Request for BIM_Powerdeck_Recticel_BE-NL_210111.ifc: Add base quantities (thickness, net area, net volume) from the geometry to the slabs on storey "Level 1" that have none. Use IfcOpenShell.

First a look at what the model holds.

```python
import ifcopenshell
import ifcopenshell.util.element
import ifcopenshell.util.unit

model = ifcopenshell.open("BIM_Powerdeck_Recticel_BE-NL_210111.ifc")
print(model.schema)
for unit_type in ("LENGTHUNIT", "AREAUNIT", "VOLUMEUNIT"):
    print(unit_type, ifcopenshell.util.unit.calculate_unit_scale(model, unit_type))
storey = next(s for s in model.by_type("IfcBuildingStorey") if s.Name == "Level 1")
slabs = [e for e in ifcopenshell.util.element.get_decomposition(storey) if e.is_a("IfcSlab")]
for e in sorted(slabs, key=lambda e: e.id()):
    print(e.id(), e.is_a(), e.Name, list(ifcopenshell.util.element.get_psets(e, qtos_only=True)), sep=" | ")
```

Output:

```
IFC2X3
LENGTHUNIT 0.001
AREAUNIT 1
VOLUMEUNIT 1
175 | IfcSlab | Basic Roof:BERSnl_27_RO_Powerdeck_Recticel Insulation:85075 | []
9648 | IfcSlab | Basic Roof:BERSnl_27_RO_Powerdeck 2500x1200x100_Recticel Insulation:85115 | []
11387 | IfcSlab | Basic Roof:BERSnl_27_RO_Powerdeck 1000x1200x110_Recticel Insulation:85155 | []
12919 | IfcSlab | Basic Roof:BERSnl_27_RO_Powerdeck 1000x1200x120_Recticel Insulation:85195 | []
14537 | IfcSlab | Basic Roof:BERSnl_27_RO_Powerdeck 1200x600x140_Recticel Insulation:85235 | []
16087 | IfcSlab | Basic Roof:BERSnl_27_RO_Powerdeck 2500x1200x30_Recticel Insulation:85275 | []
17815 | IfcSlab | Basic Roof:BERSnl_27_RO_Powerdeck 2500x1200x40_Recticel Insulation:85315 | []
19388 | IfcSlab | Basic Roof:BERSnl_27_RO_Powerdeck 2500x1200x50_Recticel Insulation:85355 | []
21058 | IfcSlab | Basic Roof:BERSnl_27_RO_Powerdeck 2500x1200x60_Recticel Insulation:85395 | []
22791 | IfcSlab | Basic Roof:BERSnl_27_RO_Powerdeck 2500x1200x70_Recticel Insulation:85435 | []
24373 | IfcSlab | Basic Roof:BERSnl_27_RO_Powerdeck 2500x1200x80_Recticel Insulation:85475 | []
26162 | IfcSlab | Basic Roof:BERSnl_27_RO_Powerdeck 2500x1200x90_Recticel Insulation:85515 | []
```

```python
import ifcopenshell
import ifcopenshell.api.pset
import ifcopenshell.geom
import ifcopenshell.util.element
import ifcopenshell.util.shape
import ifcopenshell.util.unit

model = ifcopenshell.open("BIM_Powerdeck_Recticel_BE-NL_210111.ifc")
unit_scale = ifcopenshell.util.unit.calculate_unit_scale(model)
area_scale = ifcopenshell.util.unit.calculate_unit_scale(model, "AREAUNIT")
volume_scale = ifcopenshell.util.unit.calculate_unit_scale(model, "VOLUMEUNIT")
settings = ifcopenshell.geom.settings()

storey = next(s for s in model.by_type("IfcBuildingStorey") if s.Name == "Level 1")
slabs = [e for e in ifcopenshell.util.element.get_decomposition(storey) if e.is_a("IfcSlab")]

for e in sorted(slabs, key=lambda e: e.id()):
    if ifcopenshell.util.element.get_psets(e, qtos_only=True, should_inherit=False):
        continue
    # Geometry comes back in metres, in the element's own axes.
    shape = ifcopenshell.geom.create_shape(settings, e)
    values = {
        "Width": ifcopenshell.util.shape.get_z(shape.geometry) / unit_scale,
        "NetArea": ifcopenshell.util.shape.get_footprint_area(shape.geometry) / area_scale,
        "NetVolume": ifcopenshell.util.shape.get_volume(shape.geometry) / volume_scale,
    }
    qto = ifcopenshell.api.pset.add_qto(model, product=e, name="BaseQuantities")
    ifcopenshell.api.pset.edit_qto(model, qto=qto, properties=values)
    print(e.id(), {k: round(v, 3) for k, v in values.items()})

model.write("BIM_Powerdeck_Recticel_BE-NL_210111_updated.ifc")
```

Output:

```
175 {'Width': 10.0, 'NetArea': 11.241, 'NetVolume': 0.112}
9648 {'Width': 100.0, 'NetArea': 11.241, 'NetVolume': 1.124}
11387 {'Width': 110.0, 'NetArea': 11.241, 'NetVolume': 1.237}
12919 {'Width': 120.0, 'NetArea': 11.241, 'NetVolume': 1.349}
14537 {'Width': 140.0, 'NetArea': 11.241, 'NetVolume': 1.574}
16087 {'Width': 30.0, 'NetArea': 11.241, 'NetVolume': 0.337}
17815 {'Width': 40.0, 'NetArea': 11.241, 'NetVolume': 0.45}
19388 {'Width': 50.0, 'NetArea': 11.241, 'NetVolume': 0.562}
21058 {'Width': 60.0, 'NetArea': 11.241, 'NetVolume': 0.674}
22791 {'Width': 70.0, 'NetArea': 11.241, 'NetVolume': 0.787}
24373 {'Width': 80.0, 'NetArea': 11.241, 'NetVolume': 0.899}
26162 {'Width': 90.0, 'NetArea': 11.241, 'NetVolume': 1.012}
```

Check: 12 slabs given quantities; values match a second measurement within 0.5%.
